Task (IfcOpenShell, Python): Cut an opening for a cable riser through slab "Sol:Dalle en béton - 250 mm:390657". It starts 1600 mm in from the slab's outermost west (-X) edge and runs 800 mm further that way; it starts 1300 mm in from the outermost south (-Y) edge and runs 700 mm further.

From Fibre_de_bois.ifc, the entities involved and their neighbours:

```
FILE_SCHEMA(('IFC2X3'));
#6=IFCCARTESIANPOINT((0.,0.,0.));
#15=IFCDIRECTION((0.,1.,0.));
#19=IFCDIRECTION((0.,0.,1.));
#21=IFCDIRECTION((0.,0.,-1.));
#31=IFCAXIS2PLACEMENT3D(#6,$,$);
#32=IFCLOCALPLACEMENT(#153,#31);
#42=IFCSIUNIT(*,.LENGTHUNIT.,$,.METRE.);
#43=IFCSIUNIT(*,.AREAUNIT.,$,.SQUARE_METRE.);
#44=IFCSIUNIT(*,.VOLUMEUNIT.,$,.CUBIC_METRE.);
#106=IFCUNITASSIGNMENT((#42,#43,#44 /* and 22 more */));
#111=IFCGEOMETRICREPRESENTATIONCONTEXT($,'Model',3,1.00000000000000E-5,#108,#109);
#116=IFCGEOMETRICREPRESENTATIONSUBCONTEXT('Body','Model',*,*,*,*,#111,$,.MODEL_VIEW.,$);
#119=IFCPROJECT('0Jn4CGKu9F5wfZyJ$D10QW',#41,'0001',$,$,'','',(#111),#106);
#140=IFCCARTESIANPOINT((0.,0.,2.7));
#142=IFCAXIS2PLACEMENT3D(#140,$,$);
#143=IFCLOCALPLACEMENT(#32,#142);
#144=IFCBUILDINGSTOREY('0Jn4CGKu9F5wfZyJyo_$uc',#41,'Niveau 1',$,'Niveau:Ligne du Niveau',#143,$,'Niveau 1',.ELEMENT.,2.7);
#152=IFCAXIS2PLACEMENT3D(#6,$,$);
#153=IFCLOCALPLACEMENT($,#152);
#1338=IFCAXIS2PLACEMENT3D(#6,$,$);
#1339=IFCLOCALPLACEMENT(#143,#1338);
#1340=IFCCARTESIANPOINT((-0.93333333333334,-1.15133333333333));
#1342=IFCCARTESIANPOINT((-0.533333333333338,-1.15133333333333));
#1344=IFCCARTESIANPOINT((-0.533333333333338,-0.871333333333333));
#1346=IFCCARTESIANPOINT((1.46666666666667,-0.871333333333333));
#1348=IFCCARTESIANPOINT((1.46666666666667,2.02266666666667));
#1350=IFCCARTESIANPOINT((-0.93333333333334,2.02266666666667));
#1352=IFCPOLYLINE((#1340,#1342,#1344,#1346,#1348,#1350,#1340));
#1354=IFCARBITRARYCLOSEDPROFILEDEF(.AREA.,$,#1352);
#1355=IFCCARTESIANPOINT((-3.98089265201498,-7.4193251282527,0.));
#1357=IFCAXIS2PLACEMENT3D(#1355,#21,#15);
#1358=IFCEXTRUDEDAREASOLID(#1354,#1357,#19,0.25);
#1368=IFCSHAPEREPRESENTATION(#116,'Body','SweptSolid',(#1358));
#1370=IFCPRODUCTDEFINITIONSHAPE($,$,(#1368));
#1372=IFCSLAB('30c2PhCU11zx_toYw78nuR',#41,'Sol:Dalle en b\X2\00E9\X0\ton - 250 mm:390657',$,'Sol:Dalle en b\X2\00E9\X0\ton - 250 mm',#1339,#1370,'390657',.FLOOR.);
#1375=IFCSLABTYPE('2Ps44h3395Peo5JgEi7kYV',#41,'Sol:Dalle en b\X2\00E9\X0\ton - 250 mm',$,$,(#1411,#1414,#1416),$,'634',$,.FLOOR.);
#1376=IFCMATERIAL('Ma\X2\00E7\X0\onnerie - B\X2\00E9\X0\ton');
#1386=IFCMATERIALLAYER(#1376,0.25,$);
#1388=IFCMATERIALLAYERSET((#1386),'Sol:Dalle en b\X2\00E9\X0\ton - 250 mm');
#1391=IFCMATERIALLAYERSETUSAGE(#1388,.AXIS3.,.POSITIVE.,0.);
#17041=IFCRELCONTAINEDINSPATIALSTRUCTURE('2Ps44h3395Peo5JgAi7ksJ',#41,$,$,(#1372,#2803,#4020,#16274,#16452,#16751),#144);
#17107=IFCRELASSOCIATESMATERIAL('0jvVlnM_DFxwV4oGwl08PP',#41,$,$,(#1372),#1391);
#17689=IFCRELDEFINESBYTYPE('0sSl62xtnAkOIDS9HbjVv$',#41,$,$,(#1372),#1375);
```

```python
import numpy as np
import ifcopenshell
import ifcopenshell.api.feature
import ifcopenshell.api.geometry
import ifcopenshell.api.root
import ifcopenshell.geom
import ifcopenshell.util.placement
import ifcopenshell.util.representation
import ifcopenshell.util.shape
import ifcopenshell.util.unit

model = ifcopenshell.open("Fibre_de_bois.ifc")
unit_scale = ifcopenshell.util.unit.calculate_unit_scale(model)
settings = ifcopenshell.geom.settings()


def volume(element):
    """Net volume in cubic metres, openings subtracted."""
    shape = ifcopenshell.geom.create_shape(settings, element)
    return ifcopenshell.util.shape.get_volume(shape.geometry)


slab = model.by_guid("30c2PhCU11zx_toYw78nuR")
before = volume(slab)

# Extent in the slab's own axes, in metres. The edges named are its -X and -Y sides.
slab_shape = ifcopenshell.geom.create_shape(settings, slab)
vertices = ifcopenshell.util.shape.get_vertices(slab_shape.geometry)
x_min, y_min, bottom = vertices.min(axis=0)
top = vertices[:, 2].max()

opening = ifcopenshell.api.root.create_entity(model, ifc_class="IfcOpeningElement", name="Cable riser opening")
context = ifcopenshell.util.representation.get_context(model, "Model", "Body", "MODEL_VIEW")
width, depth = 0.8, 0.7
outline = [(0.0, 0.0), (width, 0.0), (width, depth), (0.0, depth), (0.0, 0.0)]
# Overshoot both faces by 50 mm so the cut is clean.
shape = ifcopenshell.api.geometry.add_slab_representation(
    model, context=context, depth=top - bottom + 0.1, polyline=outline
)
ifcopenshell.api.geometry.assign_representation(model, product=opening, representation=shape)

matrix = ifcopenshell.util.placement.get_local_placement(slab.ObjectPlacement)
matrix[:, 3] = matrix @ np.append(np.array([x_min + 1.6, y_min + 1.3, bottom - 0.05]) / unit_scale, 1.0)
ifcopenshell.api.geometry.edit_object_placement(model, product=opening, matrix=matrix, is_si=False)
ifcopenshell.api.feature.add_feature(model, feature=opening, element=slab)

after = volume(slab)

print(f"slab volume {before:.3f} -> {after:.3f} m3")

model.write("Fibre_de_bois_v2.ifc")
```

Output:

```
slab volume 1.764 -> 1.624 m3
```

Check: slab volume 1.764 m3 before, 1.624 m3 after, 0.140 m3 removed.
